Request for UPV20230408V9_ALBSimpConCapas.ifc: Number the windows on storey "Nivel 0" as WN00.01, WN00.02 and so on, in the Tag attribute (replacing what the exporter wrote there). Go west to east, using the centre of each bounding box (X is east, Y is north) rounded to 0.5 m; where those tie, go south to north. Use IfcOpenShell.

First a look at what the model holds.

```python
import ifcopenshell
import ifcopenshell.util.element
import ifcopenshell.util.placement

model = ifcopenshell.open("UPV20230408V9_ALBSimpConCapas.ifc")
print(model.schema)
storey = next(s for s in model.by_type("IfcBuildingStorey") if s.Name == "Nivel 0")
windows = [e for e in ifcopenshell.util.element.get_decomposition(storey) if e.is_a("IfcWindow")]
for e in sorted(windows, key=lambda e: e.id()):
    origin = ifcopenshell.util.placement.get_local_placement(e.ObjectPlacement)[:3, 3]
    print(e.id(), e.Tag, e.Name, origin.round(2) + 0.0, sep=" | ")
```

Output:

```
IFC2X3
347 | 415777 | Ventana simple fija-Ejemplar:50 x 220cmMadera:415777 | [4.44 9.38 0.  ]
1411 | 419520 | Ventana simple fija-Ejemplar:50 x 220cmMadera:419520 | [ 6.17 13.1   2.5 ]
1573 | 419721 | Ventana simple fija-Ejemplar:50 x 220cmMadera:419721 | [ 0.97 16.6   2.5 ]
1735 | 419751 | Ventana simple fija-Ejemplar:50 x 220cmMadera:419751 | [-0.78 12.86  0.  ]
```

```python
import ifcopenshell
import ifcopenshell.geom
import ifcopenshell.util.element
import ifcopenshell.util.shape

model = ifcopenshell.open("UPV20230408V9_ALBSimpConCapas.ifc")
settings = ifcopenshell.geom.settings()
settings.set("use-world-coords", True)


def centre(element):
    shape = ifcopenshell.geom.create_shape(settings, element)
    return ifcopenshell.util.shape.get_bbox_centroid(shape.geometry)


storey = next(s for s in model.by_type("IfcBuildingStorey") if s.Name == "Nivel 0")
windows = [e for e in ifcopenshell.util.element.get_decomposition(storey) if e.is_a("IfcWindow")]

# Insertion points can sit at a corner or the storey origin, so sort by the geometry (in metres).
centres = {e: centre(e) for e in windows}
windows.sort(key=lambda e: (round(centres[e][0] / 0.5), centres[e][1]))

for i, e in enumerate(windows, start=1):
    number = f"WN00.{i:02d}"
    e.Tag = number
    print(e.id(), number)

model.write("UPV20230408V9_ALBSimpConCapas_v2.ifc")
```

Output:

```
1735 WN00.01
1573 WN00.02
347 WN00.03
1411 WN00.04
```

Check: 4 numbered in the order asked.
